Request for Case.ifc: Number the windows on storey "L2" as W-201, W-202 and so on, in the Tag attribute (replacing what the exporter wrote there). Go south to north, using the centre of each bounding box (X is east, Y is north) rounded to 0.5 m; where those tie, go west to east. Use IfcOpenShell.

First a look at what the model holds.

```python
import ifcopenshell
import ifcopenshell.util.element
import ifcopenshell.util.placement

model = ifcopenshell.open("Case.ifc")
print(model.schema)
storey = next(s for s in model.by_type("IfcBuildingStorey") if s.Name == "L2")
windows = [e for e in ifcopenshell.util.element.get_decomposition(storey) if e.is_a("IfcWindow")]
for e in sorted(windows, key=lambda e: e.id()):
    origin = ifcopenshell.util.placement.get_local_placement(e.ObjectPlacement)[:3, 3]
    print(e.id(), e.Tag, e.Name, origin.round(2) + 0.0, sep=" | ")
```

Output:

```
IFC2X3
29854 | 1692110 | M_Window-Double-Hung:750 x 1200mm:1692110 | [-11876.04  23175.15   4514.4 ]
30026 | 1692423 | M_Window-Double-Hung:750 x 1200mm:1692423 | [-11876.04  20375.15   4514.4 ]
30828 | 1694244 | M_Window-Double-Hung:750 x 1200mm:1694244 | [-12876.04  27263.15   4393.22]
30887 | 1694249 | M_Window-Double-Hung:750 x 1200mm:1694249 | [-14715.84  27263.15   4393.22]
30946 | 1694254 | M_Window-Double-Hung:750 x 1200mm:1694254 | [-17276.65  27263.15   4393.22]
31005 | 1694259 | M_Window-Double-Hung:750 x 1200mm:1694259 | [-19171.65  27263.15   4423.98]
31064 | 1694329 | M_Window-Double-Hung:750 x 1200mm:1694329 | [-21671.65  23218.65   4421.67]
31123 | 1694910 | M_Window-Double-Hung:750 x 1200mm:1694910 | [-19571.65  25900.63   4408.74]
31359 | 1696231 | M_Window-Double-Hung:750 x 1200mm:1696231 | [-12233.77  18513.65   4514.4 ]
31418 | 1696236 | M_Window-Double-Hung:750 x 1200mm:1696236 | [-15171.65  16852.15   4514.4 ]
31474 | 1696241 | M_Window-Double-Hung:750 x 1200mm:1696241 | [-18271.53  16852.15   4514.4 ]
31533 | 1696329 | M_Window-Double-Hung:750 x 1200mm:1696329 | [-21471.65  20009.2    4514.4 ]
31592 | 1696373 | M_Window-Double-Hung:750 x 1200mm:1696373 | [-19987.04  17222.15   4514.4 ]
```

```python
import ifcopenshell
import ifcopenshell.geom
import ifcopenshell.util.element
import ifcopenshell.util.shape

model = ifcopenshell.open("Case.ifc")
settings = ifcopenshell.geom.settings()
settings.set("use-world-coords", True)


def centre(element):
    shape = ifcopenshell.geom.create_shape(settings, element)
    return ifcopenshell.util.shape.get_bbox_centroid(shape.geometry)


storey = next(s for s in model.by_type("IfcBuildingStorey") if s.Name == "L2")
windows = [e for e in ifcopenshell.util.element.get_decomposition(storey) if e.is_a("IfcWindow")]

# Insertion points can sit at a corner or the storey origin, so sort by the geometry (in metres).
centres = {e: centre(e) for e in windows}
windows.sort(key=lambda e: (round(centres[e][1] / 0.5), centres[e][0]))

for i, e in enumerate(windows, start=1):
    number = f"W-2{i:02d}"
    e.Tag = number
    print(e.id(), number)

model.write("Case_edited.ifc")
```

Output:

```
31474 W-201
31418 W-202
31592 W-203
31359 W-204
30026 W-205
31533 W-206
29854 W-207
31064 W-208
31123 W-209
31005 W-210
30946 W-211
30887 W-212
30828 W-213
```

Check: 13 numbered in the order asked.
